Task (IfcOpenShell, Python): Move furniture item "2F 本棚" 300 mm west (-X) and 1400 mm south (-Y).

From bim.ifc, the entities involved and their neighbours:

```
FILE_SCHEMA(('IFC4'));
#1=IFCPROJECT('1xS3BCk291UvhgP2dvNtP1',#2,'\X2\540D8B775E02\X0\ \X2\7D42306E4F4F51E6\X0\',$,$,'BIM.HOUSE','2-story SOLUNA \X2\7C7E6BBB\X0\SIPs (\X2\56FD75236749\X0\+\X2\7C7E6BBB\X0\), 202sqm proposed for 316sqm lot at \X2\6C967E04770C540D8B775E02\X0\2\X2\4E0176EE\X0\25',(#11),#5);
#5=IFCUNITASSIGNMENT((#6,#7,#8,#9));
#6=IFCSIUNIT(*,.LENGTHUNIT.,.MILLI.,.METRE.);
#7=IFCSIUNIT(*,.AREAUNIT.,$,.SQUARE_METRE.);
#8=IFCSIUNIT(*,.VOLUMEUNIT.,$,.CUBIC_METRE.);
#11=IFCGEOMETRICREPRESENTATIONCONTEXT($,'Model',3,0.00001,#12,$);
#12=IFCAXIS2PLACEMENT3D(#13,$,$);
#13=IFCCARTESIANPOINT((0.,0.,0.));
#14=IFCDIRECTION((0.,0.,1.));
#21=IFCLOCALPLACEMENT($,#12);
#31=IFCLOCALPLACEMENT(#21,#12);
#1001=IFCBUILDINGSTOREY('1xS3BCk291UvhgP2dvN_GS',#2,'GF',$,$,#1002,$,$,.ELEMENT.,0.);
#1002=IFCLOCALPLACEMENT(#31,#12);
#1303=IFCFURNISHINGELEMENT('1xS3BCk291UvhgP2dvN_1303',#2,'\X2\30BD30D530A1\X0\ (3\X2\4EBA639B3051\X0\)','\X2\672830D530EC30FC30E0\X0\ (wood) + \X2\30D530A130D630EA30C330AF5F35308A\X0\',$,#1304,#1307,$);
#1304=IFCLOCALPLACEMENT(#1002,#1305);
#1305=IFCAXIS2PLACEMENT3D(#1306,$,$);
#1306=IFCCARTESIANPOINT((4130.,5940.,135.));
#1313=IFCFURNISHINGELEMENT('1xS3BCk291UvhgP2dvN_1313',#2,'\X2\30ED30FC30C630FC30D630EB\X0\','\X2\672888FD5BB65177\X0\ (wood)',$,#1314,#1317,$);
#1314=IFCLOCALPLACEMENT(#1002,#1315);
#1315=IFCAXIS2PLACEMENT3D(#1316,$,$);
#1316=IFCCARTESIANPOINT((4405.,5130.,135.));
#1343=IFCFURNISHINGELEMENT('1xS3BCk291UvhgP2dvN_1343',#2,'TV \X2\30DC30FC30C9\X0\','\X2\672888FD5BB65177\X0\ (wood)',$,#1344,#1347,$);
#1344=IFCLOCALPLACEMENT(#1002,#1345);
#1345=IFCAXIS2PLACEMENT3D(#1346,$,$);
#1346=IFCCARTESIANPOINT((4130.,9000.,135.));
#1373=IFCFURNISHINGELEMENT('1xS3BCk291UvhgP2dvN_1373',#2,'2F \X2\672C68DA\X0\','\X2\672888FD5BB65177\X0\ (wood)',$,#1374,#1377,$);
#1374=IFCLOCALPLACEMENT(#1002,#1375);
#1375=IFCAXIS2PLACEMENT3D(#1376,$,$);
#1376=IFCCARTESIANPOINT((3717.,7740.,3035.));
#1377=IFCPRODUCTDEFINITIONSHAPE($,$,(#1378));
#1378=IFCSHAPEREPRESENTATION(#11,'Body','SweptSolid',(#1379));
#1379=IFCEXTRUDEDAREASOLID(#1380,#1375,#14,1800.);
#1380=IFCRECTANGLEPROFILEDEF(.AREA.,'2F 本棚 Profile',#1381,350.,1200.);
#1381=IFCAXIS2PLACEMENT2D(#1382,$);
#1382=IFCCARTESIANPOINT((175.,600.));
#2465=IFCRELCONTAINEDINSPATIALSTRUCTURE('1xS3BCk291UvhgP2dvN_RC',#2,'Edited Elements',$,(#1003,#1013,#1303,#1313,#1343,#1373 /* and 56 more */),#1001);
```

```python
import ifcopenshell
import ifcopenshell.api.geometry
import ifcopenshell.util.placement

model = ifcopenshell.open("bim.ifc")

item = model.by_id(1373)
matrix = ifcopenshell.util.placement.get_local_placement(item.ObjectPlacement)
matrix[0, 3] -= 300.0
matrix[1, 3] -= 1400.0
ifcopenshell.api.geometry.edit_object_placement(model, product=item, matrix=matrix, is_si=False)

print(ifcopenshell.util.placement.get_local_placement(item.ObjectPlacement).round(3) + 0.0)

model.write("bim_updated.ifc")
```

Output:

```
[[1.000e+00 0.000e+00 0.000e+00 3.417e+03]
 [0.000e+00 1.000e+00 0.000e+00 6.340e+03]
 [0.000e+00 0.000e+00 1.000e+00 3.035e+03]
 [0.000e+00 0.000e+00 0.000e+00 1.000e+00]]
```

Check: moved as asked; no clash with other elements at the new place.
